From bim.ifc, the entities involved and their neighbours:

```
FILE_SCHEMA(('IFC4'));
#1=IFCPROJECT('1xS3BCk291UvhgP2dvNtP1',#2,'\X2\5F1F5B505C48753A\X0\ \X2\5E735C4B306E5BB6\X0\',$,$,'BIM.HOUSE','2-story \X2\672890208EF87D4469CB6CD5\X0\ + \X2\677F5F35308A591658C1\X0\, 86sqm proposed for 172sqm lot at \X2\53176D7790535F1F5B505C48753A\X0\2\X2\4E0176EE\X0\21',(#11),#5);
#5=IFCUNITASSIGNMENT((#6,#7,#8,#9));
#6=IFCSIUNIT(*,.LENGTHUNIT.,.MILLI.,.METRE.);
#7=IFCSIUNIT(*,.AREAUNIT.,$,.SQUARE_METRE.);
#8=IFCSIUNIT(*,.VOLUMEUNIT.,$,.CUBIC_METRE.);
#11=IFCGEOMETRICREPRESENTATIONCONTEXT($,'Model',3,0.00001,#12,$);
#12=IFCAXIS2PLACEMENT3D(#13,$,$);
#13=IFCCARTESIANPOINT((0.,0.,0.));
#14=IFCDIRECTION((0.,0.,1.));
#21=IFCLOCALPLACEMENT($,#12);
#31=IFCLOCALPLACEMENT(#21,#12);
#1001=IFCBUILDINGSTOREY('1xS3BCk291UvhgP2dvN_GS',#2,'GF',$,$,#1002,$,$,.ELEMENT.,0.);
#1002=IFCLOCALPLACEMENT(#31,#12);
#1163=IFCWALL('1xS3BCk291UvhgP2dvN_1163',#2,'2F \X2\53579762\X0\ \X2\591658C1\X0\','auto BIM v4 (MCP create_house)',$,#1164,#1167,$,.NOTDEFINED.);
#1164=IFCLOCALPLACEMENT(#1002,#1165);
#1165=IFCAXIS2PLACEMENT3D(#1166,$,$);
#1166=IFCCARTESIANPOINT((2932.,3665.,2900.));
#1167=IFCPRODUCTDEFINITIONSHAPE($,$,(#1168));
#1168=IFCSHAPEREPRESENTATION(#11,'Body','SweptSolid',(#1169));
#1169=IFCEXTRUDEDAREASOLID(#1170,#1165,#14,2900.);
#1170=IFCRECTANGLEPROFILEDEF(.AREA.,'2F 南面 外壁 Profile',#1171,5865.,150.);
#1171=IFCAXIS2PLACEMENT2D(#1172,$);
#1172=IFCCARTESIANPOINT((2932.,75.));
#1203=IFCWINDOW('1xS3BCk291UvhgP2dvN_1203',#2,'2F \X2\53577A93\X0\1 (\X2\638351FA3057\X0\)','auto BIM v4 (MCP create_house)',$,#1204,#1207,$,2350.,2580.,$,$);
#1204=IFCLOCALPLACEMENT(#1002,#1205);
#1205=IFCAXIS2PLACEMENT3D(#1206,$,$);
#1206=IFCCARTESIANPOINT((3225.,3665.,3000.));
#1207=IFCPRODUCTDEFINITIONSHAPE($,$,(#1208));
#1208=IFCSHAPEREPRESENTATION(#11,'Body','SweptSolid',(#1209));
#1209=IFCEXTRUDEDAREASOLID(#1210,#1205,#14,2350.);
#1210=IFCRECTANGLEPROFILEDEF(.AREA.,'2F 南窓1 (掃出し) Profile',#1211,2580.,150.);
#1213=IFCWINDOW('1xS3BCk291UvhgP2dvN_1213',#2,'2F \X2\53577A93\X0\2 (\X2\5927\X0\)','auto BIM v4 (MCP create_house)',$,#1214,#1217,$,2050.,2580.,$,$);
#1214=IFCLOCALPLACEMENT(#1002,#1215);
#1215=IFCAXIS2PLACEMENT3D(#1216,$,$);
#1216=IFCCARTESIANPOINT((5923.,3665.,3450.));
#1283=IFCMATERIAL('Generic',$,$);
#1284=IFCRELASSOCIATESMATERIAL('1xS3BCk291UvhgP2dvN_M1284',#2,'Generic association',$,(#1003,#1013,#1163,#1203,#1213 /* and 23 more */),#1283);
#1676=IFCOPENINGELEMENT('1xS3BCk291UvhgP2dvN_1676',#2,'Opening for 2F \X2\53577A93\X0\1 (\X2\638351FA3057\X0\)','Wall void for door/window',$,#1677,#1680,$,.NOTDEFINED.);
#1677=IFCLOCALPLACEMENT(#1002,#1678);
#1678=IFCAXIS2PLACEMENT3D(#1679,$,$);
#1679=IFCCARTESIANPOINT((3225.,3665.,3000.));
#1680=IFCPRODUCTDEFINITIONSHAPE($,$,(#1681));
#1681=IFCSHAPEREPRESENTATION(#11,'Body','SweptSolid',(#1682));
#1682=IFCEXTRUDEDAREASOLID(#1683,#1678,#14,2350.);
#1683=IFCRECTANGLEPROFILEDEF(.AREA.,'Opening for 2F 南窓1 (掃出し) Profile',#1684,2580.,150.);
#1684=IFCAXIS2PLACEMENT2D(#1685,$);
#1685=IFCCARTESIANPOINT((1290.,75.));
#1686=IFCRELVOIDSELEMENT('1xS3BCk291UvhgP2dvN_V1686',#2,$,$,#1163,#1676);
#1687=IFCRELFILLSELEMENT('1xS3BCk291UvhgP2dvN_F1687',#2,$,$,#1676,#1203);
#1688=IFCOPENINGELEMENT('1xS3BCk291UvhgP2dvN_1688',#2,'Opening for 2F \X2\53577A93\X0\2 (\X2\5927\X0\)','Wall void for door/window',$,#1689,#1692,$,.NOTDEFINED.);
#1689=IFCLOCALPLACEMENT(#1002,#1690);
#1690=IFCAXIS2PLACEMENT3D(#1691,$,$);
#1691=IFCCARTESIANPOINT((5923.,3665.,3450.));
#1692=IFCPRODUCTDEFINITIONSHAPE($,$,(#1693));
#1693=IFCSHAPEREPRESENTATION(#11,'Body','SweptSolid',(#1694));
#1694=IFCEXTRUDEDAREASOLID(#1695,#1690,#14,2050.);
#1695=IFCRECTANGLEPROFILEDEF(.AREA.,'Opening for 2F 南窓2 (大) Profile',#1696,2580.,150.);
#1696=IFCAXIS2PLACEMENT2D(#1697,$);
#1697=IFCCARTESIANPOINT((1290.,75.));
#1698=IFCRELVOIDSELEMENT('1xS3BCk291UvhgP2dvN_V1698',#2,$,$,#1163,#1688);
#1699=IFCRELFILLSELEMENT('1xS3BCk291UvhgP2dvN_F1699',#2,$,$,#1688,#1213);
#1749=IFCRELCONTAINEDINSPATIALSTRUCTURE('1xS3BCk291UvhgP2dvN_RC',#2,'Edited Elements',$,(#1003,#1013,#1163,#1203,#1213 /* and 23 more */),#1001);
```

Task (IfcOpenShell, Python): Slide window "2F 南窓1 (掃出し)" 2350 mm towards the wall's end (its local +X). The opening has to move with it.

```python
import ifcopenshell
import ifcopenshell.api.geometry
import ifcopenshell.util.placement
import ifcopenshell.util.unit

model = ifcopenshell.open("bim.ifc")
unit_scale = ifcopenshell.util.unit.calculate_unit_scale(model)

window = model.by_guid("1xS3BCk291UvhgP2dvN_1203")
opening = window.FillsVoids[0].RelatingOpeningElement
wall = opening.VoidsElements[0].RelatingBuildingElement

wall_matrix = ifcopenshell.util.placement.get_local_placement(wall.ObjectPlacement)
shift = wall_matrix[:3, 0] * 2.35 / unit_scale
before = ifcopenshell.util.placement.get_local_placement(window.ObjectPlacement)[:3, 3].copy()

# The window is not placed relative to its opening, so move both.
for product in (opening, window):
    matrix = ifcopenshell.util.placement.get_local_placement(product.ObjectPlacement)
    matrix[:3, 3] += shift
    ifcopenshell.api.geometry.edit_object_placement(model, product=product, matrix=matrix, is_si=False)

after = ifcopenshell.util.placement.get_local_placement(window.ObjectPlacement)[:3, 3]
print("window moved by", (after - before).round(3) + 0.0)

model.write("bim-out.ifc")
```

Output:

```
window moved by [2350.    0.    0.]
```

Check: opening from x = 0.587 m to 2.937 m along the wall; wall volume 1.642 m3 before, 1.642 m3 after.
